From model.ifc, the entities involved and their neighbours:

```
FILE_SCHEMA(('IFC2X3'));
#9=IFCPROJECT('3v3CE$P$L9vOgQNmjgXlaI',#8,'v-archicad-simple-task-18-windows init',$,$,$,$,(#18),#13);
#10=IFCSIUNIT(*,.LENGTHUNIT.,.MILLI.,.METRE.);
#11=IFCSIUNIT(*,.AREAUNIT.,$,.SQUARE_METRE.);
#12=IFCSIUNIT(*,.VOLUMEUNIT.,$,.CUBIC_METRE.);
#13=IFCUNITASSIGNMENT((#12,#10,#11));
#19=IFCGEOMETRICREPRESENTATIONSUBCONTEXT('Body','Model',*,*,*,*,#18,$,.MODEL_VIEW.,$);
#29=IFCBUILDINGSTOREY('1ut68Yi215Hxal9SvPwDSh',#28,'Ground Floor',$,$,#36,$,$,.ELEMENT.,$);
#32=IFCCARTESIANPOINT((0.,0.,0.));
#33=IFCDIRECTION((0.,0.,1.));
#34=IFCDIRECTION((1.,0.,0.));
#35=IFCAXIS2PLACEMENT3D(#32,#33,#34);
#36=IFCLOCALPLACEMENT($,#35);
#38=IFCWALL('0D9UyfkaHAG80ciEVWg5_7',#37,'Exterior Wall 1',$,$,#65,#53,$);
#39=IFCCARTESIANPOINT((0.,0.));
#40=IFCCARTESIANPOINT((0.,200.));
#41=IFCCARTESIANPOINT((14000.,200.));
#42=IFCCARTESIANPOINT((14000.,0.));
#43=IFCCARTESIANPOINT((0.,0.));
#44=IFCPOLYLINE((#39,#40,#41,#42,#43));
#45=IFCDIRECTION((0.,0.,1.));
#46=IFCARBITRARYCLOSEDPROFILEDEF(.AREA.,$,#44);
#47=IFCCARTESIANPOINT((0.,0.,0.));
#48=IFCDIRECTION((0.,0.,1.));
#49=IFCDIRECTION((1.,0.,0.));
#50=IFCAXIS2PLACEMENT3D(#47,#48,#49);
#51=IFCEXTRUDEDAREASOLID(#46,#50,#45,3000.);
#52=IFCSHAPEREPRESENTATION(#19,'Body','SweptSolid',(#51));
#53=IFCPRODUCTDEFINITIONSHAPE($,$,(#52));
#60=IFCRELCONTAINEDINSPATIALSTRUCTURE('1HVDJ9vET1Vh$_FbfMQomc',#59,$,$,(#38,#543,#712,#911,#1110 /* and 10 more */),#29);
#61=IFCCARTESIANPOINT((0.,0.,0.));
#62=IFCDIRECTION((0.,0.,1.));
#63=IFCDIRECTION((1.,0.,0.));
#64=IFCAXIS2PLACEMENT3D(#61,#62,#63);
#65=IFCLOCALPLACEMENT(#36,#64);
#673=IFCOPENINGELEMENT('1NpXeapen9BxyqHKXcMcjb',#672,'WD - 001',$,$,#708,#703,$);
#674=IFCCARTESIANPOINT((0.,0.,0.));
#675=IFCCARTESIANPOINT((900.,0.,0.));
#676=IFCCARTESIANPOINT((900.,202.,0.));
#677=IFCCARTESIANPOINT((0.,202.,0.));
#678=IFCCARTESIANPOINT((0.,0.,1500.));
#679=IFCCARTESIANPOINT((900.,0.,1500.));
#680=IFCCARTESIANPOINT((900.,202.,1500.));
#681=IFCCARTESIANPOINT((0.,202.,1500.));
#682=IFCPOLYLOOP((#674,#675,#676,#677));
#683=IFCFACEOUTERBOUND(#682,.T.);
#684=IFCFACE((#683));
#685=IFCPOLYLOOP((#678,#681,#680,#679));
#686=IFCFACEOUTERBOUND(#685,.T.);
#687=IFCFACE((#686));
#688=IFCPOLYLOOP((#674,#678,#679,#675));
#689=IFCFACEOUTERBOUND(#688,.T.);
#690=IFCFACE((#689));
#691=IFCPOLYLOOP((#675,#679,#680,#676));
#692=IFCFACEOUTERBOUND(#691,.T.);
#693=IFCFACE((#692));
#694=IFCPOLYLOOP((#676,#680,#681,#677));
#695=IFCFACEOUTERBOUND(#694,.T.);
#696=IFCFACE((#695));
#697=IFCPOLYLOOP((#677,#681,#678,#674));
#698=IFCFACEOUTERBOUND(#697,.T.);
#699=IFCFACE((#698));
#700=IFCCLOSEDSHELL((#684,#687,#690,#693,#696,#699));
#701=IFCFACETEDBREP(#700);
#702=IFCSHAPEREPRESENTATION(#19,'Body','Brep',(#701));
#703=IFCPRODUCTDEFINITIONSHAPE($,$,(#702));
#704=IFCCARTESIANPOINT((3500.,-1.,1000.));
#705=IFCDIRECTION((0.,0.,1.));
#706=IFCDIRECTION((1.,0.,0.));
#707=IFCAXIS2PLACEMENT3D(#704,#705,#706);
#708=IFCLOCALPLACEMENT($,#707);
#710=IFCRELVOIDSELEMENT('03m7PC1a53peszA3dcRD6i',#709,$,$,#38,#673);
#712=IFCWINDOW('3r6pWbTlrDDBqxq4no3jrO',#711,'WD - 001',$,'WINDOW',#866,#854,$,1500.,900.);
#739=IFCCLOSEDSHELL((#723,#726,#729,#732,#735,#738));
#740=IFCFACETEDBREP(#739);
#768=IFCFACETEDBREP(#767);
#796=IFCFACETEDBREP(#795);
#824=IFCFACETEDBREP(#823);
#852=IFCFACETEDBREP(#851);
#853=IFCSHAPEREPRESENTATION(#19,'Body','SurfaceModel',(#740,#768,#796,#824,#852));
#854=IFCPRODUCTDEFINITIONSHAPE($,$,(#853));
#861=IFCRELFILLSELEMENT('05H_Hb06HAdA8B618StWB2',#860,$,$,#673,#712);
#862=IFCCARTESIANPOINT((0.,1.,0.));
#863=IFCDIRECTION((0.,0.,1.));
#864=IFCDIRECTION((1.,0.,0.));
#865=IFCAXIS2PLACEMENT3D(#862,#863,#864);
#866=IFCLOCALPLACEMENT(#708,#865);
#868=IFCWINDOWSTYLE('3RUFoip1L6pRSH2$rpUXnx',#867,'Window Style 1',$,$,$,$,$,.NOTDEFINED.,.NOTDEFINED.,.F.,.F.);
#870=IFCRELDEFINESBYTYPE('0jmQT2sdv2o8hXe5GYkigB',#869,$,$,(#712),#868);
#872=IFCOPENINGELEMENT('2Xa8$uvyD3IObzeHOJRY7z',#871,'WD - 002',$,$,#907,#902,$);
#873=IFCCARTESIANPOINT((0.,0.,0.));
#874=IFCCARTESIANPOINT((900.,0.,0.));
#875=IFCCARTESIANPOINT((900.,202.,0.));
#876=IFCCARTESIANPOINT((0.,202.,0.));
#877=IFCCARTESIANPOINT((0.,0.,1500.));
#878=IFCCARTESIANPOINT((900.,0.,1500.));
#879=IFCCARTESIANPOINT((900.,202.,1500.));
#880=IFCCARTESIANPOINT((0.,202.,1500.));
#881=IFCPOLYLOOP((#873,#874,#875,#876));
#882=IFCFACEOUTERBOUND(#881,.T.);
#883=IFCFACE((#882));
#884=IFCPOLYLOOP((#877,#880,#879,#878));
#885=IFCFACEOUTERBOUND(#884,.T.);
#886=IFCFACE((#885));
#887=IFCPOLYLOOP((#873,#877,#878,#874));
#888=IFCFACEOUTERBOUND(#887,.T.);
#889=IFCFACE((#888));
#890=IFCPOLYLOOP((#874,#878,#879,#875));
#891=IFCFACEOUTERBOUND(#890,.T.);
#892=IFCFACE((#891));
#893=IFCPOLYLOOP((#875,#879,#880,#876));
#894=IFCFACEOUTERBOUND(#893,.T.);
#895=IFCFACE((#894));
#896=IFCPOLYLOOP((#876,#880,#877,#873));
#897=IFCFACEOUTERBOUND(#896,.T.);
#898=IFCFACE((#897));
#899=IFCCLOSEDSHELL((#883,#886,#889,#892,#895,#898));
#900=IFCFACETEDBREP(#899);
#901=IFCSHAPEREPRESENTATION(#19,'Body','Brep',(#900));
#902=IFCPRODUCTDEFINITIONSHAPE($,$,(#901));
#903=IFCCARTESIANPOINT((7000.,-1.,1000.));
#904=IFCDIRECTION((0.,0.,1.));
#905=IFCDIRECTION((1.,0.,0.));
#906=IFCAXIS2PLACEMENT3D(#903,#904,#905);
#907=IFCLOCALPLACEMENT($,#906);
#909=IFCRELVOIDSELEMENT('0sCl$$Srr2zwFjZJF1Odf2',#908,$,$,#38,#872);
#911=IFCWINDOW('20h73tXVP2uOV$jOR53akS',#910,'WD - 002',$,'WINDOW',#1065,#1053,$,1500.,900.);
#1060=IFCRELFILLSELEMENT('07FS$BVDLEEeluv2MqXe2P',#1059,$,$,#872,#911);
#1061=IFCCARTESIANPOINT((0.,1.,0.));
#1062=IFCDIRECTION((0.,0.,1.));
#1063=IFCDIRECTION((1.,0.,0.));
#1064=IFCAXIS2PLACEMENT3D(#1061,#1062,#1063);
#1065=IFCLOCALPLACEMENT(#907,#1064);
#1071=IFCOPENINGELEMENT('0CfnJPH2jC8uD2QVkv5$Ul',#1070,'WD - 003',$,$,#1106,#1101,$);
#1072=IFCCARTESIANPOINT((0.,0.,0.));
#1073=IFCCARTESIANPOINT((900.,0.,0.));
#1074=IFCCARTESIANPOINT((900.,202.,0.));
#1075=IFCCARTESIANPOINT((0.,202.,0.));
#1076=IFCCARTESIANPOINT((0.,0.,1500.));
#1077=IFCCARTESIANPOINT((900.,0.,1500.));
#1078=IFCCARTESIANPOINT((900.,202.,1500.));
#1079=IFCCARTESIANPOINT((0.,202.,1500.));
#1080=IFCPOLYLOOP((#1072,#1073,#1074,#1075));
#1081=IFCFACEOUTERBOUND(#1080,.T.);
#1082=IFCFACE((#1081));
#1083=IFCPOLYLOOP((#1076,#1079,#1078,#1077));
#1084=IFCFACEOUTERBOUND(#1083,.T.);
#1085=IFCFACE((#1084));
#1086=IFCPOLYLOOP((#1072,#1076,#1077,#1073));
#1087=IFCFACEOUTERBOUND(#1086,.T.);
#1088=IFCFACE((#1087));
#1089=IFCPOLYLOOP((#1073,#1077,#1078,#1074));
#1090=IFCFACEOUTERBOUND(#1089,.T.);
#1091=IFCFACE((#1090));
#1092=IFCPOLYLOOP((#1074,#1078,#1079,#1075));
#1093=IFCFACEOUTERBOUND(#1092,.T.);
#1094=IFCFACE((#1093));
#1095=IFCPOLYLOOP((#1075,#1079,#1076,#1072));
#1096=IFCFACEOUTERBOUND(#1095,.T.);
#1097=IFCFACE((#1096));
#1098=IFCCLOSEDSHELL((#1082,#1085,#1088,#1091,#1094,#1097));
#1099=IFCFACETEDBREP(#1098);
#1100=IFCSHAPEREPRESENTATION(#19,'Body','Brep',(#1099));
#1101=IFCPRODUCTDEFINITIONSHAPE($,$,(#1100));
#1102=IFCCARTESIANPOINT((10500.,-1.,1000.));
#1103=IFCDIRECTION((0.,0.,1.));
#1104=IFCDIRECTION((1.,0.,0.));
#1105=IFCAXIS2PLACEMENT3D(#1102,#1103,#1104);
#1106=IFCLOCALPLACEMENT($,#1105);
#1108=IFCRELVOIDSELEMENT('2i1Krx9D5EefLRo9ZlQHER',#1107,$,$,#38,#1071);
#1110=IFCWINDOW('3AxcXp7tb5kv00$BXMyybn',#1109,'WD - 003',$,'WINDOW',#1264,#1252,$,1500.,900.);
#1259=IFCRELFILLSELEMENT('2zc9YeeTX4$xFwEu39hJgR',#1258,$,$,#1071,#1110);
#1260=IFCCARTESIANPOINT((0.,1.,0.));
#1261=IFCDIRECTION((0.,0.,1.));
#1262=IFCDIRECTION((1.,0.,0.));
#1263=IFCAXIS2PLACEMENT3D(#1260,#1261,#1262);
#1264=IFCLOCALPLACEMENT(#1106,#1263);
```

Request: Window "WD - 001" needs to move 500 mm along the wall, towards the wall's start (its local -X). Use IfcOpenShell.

```python
import ifcopenshell
import ifcopenshell.api.geometry
import ifcopenshell.util.placement
import ifcopenshell.util.unit

model = ifcopenshell.open("model.ifc")
unit_scale = ifcopenshell.util.unit.calculate_unit_scale(model)

window = model.by_guid("3r6pWbTlrDDBqxq4no3jrO")
opening = window.FillsVoids[0].RelatingOpeningElement
wall = opening.VoidsElements[0].RelatingBuildingElement

wall_matrix = ifcopenshell.util.placement.get_local_placement(wall.ObjectPlacement)
shift = wall_matrix[:3, 0] * -0.5 / unit_scale
before = ifcopenshell.util.placement.get_local_placement(window.ObjectPlacement)[:3, 3].copy()

# The window is placed relative to its opening, so it follows when the opening moves.
matrix = ifcopenshell.util.placement.get_local_placement(opening.ObjectPlacement)
matrix[:3, 3] += shift
ifcopenshell.api.geometry.edit_object_placement(
    model, product=opening, matrix=matrix, is_si=False, should_transform_children=True
)

after = ifcopenshell.util.placement.get_local_placement(window.ObjectPlacement)[:3, 3]
print("window moved by", (after - before).round(3) + 0.0)

model.write("model_rev.ifc")
```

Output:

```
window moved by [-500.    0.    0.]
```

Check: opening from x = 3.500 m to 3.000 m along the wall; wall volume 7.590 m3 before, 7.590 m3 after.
